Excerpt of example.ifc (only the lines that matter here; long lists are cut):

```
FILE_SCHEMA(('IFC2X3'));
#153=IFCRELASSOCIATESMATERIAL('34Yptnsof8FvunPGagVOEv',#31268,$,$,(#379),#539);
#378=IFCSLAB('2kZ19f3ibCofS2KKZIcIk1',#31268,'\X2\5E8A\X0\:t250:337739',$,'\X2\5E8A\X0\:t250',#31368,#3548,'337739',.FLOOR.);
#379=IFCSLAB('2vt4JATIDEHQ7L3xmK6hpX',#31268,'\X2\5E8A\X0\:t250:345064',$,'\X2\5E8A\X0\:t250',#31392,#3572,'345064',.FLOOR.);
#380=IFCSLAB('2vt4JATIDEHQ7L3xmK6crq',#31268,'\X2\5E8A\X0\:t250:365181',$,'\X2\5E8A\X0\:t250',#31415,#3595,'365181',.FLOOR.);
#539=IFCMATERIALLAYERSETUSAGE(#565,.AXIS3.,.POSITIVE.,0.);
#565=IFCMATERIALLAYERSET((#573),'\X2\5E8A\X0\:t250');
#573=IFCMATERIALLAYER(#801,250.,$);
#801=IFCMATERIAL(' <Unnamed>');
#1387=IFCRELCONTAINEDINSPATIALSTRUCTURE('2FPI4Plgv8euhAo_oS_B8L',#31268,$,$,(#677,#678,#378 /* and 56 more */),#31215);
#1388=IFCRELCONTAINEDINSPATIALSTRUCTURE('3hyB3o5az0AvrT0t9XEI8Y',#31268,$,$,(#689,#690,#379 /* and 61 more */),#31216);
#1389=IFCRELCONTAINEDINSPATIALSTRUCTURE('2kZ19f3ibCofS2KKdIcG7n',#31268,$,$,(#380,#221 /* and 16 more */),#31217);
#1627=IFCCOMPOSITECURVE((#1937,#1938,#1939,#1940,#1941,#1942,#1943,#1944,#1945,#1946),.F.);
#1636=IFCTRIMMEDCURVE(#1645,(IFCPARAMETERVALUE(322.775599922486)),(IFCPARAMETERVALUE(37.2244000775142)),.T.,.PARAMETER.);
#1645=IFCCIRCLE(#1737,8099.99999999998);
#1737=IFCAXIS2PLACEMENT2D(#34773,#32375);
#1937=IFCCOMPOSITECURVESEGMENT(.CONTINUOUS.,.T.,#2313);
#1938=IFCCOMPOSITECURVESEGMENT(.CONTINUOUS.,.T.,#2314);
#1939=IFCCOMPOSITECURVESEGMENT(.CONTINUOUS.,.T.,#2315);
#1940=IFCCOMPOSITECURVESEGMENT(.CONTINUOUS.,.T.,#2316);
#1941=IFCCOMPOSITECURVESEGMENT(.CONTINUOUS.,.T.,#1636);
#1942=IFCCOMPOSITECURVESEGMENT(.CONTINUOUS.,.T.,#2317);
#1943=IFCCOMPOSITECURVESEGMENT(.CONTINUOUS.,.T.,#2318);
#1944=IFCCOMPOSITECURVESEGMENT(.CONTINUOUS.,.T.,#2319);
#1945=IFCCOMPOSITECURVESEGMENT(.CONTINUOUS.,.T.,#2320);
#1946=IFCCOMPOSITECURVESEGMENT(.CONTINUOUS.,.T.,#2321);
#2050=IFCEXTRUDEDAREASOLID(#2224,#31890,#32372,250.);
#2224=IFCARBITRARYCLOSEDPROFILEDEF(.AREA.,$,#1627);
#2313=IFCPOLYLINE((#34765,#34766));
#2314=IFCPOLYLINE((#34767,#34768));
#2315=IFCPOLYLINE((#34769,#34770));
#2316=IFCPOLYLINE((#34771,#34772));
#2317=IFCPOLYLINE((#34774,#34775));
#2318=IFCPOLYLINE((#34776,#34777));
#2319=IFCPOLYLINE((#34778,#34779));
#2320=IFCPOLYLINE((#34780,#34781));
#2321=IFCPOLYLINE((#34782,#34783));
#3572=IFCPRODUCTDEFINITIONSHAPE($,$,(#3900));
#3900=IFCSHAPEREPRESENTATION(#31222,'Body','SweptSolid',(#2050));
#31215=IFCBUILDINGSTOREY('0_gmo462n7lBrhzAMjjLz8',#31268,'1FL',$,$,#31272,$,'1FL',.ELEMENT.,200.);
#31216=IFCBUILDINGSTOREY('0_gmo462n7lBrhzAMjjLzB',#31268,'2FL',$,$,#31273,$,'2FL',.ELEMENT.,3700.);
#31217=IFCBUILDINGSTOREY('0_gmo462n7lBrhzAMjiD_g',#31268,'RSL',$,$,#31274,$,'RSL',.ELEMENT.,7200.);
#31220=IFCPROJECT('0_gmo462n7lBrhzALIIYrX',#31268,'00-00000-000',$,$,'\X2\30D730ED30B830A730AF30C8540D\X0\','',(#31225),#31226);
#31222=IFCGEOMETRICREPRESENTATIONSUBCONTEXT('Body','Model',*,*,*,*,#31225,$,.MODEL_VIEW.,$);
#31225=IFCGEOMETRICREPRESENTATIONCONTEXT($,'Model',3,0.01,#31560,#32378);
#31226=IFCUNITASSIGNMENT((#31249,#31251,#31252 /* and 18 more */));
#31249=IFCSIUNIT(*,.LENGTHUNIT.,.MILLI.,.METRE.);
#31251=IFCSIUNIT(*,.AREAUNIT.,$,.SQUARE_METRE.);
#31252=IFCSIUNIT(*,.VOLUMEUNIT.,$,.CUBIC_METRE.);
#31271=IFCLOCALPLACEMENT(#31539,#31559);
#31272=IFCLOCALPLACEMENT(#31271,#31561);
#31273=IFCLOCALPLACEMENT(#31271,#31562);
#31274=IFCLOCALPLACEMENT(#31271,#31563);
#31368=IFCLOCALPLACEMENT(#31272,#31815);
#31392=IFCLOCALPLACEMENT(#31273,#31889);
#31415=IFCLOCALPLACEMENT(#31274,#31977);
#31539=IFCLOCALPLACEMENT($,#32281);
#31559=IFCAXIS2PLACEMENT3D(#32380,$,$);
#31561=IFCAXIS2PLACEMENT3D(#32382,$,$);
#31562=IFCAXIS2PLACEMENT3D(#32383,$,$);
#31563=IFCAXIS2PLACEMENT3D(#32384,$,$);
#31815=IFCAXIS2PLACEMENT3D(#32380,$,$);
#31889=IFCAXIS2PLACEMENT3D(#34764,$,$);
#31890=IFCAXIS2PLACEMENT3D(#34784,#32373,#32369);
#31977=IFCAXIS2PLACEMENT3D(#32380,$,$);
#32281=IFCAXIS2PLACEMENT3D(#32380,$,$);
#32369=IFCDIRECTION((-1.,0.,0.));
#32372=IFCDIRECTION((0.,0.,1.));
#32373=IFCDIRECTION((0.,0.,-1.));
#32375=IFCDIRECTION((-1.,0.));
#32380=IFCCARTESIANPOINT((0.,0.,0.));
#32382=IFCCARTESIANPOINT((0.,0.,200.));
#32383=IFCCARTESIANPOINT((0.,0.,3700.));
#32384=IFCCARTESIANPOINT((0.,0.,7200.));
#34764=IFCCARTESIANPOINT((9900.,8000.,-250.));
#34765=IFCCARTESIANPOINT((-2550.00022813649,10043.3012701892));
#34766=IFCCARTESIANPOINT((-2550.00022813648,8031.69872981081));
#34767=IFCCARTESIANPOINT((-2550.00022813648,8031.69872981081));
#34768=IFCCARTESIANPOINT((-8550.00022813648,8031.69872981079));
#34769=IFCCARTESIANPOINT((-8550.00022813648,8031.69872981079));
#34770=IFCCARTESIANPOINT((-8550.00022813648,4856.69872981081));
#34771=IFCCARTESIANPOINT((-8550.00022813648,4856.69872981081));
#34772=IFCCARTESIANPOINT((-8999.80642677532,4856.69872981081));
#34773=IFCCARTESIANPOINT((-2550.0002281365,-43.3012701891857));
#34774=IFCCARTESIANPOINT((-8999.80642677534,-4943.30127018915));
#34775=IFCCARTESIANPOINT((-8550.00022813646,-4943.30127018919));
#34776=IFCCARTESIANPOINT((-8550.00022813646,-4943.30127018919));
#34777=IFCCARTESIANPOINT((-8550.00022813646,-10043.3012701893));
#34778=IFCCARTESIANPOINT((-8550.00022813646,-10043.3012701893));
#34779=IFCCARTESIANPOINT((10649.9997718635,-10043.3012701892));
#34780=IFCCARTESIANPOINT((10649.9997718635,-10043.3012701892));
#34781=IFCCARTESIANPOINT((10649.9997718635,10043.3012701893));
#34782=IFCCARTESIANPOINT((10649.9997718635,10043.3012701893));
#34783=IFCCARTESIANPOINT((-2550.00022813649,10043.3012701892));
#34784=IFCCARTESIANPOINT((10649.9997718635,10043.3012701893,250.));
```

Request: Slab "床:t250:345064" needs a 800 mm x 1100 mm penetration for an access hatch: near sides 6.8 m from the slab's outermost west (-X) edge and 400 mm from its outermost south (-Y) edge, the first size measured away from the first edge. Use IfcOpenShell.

```python
import numpy as np
import ifcopenshell
import ifcopenshell.api.feature
import ifcopenshell.api.geometry
import ifcopenshell.api.root
import ifcopenshell.geom
import ifcopenshell.util.placement
import ifcopenshell.util.representation
import ifcopenshell.util.shape
import ifcopenshell.util.unit

model = ifcopenshell.open("example.ifc")
unit_scale = ifcopenshell.util.unit.calculate_unit_scale(model)
settings = ifcopenshell.geom.settings()


def volume(element):
    """Net volume in cubic metres, openings subtracted."""
    shape = ifcopenshell.geom.create_shape(settings, element)
    return ifcopenshell.util.shape.get_volume(shape.geometry)


slab = model.by_guid("2vt4JATIDEHQ7L3xmK6hpX")
before = volume(slab)

# Extent in the slab's own axes, in metres. The edges named are its -X and -Y sides.
slab_shape = ifcopenshell.geom.create_shape(settings, slab)
vertices = ifcopenshell.util.shape.get_vertices(slab_shape.geometry)
x_min, y_min, bottom = vertices.min(axis=0)
top = vertices[:, 2].max()

opening = ifcopenshell.api.root.create_entity(model, ifc_class="IfcOpeningElement", name="Access hatch opening")
context = ifcopenshell.util.representation.get_context(model, "Model", "Body", "MODEL_VIEW")
width, depth = 0.8, 1.1
outline = [(0.0, 0.0), (width, 0.0), (width, depth), (0.0, depth), (0.0, 0.0)]
# Overshoot both faces by 50 mm so the cut is clean.
shape = ifcopenshell.api.geometry.add_slab_representation(
    model, context=context, depth=top - bottom + 0.1, polyline=outline
)
ifcopenshell.api.geometry.assign_representation(model, product=opening, representation=shape)

matrix = ifcopenshell.util.placement.get_local_placement(slab.ObjectPlacement)
matrix[:, 3] = matrix @ np.append(np.array([x_min + 6.8, y_min + 0.4, bottom - 0.05]) / unit_scale, 1.0)
ifcopenshell.api.geometry.edit_object_placement(model, product=opening, matrix=matrix, is_si=False)
ifcopenshell.api.feature.add_feature(model, feature=opening, element=slab)

after = volume(slab)

print(f"slab volume {before:.3f} -> {after:.3f} m3")

model.write("example_rev.ifc")
```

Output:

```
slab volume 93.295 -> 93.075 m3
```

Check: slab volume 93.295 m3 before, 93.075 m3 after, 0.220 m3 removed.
